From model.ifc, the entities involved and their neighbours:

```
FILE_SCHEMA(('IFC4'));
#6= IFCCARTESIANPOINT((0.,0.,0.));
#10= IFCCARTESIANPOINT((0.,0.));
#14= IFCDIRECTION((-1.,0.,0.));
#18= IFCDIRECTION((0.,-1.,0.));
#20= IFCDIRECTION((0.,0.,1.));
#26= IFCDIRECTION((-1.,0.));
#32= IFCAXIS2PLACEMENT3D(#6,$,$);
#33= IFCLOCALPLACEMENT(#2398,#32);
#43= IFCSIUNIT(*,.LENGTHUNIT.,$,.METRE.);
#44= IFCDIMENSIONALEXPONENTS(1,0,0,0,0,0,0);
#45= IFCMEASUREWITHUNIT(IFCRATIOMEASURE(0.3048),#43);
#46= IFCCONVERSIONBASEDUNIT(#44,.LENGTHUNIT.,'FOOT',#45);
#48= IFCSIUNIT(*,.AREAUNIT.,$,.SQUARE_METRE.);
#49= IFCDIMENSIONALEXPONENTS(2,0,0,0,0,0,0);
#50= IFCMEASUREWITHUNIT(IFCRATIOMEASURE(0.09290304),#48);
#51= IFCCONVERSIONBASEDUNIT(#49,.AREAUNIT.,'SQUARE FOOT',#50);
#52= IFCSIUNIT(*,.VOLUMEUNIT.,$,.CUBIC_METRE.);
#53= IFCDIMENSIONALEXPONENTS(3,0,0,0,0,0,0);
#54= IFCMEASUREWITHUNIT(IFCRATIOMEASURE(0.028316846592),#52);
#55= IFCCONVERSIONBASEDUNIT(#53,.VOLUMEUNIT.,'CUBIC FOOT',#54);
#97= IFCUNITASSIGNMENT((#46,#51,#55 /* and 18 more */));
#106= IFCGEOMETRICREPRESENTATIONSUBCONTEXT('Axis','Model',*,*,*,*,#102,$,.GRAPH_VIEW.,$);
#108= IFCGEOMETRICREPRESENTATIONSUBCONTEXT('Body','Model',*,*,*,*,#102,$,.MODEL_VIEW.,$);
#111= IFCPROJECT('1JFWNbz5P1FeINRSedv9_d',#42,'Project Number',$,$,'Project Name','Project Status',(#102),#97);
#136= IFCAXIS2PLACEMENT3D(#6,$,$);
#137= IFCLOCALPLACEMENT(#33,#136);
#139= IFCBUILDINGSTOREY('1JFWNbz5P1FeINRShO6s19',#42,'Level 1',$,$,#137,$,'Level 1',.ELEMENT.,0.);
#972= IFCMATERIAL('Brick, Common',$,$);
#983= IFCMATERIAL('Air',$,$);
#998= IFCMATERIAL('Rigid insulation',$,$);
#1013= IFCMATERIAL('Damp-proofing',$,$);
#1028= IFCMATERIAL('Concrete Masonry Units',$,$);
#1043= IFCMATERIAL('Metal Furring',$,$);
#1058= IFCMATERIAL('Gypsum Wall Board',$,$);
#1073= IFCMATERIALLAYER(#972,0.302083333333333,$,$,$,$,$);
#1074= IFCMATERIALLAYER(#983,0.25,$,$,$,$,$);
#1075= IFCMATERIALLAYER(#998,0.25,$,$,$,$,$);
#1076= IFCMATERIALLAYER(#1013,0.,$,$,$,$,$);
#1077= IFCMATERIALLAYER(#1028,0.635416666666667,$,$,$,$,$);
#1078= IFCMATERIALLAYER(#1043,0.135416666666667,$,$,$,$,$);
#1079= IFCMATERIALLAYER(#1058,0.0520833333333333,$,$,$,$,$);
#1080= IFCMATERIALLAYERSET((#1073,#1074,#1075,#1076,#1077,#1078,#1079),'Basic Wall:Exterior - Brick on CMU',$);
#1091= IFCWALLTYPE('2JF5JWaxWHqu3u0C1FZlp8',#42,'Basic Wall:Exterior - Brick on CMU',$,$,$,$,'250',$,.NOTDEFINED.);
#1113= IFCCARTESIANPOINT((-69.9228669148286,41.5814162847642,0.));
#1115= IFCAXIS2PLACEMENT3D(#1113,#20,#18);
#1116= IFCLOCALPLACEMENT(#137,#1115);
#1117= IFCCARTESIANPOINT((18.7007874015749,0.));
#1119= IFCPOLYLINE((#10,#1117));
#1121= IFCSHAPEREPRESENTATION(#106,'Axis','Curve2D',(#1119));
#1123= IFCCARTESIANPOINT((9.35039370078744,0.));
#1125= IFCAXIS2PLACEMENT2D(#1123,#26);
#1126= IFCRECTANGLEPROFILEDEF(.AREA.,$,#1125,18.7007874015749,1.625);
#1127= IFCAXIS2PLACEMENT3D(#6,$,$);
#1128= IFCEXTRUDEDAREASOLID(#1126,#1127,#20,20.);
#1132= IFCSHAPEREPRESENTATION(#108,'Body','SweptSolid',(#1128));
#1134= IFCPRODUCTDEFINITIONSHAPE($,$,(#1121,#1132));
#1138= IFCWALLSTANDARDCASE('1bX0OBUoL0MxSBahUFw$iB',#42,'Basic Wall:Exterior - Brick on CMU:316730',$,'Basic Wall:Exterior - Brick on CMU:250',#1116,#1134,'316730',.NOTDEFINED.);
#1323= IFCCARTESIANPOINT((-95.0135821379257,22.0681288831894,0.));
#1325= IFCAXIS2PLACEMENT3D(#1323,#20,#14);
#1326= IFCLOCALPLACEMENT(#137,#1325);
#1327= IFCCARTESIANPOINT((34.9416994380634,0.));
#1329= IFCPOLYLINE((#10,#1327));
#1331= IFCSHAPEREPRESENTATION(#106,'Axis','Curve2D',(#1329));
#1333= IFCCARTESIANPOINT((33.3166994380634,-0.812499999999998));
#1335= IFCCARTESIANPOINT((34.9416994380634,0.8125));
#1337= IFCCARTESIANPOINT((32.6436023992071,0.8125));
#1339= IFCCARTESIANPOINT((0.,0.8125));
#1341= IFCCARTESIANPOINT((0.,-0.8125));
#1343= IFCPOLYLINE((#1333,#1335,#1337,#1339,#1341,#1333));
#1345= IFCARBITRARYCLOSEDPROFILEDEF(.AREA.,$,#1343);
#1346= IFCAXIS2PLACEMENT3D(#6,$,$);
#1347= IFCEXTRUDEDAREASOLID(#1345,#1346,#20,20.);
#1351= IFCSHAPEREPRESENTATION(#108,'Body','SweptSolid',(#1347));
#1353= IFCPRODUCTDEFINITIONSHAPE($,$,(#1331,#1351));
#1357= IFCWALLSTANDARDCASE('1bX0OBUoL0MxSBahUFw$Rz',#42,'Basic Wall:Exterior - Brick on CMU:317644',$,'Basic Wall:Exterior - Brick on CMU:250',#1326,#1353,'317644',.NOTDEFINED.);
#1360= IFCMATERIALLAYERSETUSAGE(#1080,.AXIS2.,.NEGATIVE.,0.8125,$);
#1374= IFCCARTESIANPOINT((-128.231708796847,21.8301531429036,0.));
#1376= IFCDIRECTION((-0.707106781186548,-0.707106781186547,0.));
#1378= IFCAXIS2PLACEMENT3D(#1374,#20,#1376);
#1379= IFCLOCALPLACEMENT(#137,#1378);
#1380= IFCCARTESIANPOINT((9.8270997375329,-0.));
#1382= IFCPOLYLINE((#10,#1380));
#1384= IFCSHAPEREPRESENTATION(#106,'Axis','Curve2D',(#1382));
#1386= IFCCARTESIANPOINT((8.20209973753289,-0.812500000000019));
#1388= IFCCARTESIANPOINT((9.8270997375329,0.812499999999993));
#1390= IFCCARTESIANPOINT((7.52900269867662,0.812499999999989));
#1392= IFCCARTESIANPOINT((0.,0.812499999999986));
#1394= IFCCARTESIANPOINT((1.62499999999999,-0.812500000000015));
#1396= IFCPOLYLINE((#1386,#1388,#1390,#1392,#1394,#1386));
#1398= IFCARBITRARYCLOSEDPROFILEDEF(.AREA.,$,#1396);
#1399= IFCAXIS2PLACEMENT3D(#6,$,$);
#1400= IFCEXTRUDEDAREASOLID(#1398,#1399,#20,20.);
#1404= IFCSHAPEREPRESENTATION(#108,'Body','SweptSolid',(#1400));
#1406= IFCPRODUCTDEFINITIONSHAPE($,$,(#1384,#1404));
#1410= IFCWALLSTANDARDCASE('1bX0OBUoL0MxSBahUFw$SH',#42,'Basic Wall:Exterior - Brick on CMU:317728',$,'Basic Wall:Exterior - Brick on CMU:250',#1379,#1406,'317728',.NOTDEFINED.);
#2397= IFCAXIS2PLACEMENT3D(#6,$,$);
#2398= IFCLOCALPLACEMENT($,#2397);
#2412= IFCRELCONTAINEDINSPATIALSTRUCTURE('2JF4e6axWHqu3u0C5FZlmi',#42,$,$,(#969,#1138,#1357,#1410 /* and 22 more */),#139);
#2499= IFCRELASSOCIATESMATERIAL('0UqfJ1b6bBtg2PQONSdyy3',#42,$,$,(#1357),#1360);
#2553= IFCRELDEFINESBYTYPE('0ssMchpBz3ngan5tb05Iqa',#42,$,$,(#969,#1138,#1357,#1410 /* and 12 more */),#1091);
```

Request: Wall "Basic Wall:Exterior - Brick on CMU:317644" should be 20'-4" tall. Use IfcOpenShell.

```python
import ifcopenshell
import ifcopenshell.geom
import ifcopenshell.util.representation
import ifcopenshell.util.shape
import ifcopenshell.util.unit

model = ifcopenshell.open("model.ifc")
unit_scale = ifcopenshell.util.unit.calculate_unit_scale(model)
settings = ifcopenshell.geom.settings()


def volume(element):
    """Net volume in cubic metres, openings subtracted."""
    shape = ifcopenshell.geom.create_shape(settings, element)
    return ifcopenshell.util.shape.get_volume(shape.geometry)


wall = model.by_guid("1bX0OBUoL0MxSBahUFw$Rz")
before = volume(wall)

body = ifcopenshell.util.representation.get_representation(wall, "Model", "Body")
solid = body.Items[0]
old_height = solid.Depth
solid.Depth = 244 * 0.0254 / unit_scale
after = volume(wall)

print(f"height {old_height:g} -> {solid.Depth:g}, volume {before:.3f} -> {after:.3f} m3")

model.write("model_edited.ifc")
```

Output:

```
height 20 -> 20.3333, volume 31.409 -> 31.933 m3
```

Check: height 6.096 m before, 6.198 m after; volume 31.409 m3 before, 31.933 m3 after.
